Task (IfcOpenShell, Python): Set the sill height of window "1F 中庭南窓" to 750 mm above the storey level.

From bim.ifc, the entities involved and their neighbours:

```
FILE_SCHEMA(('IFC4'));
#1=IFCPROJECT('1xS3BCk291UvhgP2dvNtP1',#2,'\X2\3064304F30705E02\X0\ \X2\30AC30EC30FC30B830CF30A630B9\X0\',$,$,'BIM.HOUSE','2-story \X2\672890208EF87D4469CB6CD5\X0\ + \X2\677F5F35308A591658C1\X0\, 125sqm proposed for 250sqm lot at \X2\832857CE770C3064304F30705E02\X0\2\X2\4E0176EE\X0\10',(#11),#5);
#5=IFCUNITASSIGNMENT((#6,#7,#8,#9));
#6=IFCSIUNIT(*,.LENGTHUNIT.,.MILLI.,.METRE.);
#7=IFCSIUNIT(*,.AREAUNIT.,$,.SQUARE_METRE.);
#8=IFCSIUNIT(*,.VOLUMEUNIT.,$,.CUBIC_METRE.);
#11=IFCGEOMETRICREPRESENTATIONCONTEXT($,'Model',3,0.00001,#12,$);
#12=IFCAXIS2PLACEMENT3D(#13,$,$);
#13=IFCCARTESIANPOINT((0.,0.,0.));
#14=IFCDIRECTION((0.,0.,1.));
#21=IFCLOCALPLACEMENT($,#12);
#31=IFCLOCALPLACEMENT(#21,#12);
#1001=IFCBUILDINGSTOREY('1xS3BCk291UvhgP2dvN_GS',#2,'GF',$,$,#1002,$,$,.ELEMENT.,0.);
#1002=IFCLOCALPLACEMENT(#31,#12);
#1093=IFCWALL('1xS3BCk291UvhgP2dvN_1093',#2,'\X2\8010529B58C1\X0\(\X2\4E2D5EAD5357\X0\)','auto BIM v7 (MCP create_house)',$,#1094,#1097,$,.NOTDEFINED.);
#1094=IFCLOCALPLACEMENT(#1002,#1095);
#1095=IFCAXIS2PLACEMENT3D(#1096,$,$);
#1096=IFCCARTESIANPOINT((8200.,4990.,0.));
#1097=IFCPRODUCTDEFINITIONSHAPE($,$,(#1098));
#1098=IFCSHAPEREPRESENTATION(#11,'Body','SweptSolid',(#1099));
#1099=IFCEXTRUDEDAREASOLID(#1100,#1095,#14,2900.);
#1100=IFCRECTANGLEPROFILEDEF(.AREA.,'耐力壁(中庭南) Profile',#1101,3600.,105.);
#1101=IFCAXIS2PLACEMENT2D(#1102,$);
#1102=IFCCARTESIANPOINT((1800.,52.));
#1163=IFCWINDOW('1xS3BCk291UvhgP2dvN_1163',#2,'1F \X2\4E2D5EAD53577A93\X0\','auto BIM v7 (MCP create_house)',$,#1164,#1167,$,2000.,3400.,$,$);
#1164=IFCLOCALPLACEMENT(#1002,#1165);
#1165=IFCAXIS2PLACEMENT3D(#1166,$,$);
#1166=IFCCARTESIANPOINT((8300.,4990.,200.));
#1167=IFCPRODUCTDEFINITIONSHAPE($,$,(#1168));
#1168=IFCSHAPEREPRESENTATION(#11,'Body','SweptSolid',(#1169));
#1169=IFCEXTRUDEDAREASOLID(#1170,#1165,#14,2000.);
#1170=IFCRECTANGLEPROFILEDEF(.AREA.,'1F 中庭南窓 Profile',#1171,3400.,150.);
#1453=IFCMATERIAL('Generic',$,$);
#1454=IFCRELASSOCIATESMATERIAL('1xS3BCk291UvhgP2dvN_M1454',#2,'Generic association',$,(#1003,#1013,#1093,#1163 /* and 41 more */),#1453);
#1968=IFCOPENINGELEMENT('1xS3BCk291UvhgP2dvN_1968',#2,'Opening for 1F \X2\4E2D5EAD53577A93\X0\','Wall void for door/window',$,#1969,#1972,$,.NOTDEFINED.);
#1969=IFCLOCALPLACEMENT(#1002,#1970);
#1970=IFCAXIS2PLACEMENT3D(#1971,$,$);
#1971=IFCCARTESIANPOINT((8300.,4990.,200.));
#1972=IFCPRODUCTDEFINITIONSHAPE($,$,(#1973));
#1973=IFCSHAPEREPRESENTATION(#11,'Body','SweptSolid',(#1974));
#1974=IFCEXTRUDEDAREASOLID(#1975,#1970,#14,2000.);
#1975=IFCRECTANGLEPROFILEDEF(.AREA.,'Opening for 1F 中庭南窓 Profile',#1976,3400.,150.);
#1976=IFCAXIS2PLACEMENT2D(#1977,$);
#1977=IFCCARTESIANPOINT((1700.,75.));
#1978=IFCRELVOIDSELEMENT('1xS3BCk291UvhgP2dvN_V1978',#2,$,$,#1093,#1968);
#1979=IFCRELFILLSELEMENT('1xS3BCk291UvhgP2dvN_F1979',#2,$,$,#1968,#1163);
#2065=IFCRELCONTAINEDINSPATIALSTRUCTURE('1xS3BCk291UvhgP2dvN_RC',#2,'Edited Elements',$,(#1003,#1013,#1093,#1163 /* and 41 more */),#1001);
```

```python
import numpy as np
import ifcopenshell
import ifcopenshell.api.geometry
import ifcopenshell.geom
import ifcopenshell.util.element
import ifcopenshell.util.placement
import ifcopenshell.util.shape
import ifcopenshell.util.unit

model = ifcopenshell.open("bim.ifc")
unit_scale = ifcopenshell.util.unit.calculate_unit_scale(model)

window = model.by_id(1163)
opening = window.FillsVoids[0].RelatingOpeningElement
storey = ifcopenshell.util.element.get_container(window, ifc_class="IfcBuildingStorey")
level = ifcopenshell.util.placement.get_local_placement(storey.ObjectPlacement)[2, 3]

# The opening's origin need not be at the sill, so measure its lowest point.
shape = ifcopenshell.geom.create_shape(ifcopenshell.geom.settings(), opening)
bottom = ifcopenshell.util.shape.get_shape_bottom_elevation(shape, shape.geometry) / unit_scale
dz = level + 0.75 / unit_scale - bottom

shift = np.array([0.0, 0.0, dz])
# The window is not placed relative to its opening, so move both.
for product in (opening, window):
    matrix = ifcopenshell.util.placement.get_local_placement(product.ObjectPlacement)
    matrix[:3, 3] += shift
    ifcopenshell.api.geometry.edit_object_placement(model, product=product, matrix=matrix, is_si=False)

print(f"moved by {dz * unit_scale:+.3f} m")

model.write("bim_updated.ifc")
```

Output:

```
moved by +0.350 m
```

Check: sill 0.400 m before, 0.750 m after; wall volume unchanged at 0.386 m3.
